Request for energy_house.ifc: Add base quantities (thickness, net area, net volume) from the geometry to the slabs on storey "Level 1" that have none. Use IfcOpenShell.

First a look at what the model holds.

```python
import ifcopenshell
import ifcopenshell.util.element
import ifcopenshell.util.unit

model = ifcopenshell.open("energy_house.ifc")
print(model.schema)
for unit_type in ("LENGTHUNIT", "AREAUNIT", "VOLUMEUNIT"):
    print(unit_type, ifcopenshell.util.unit.calculate_unit_scale(model, unit_type))
storey = next(s for s in model.by_type("IfcBuildingStorey") if s.Name == "Level 1")
slabs = [e for e in ifcopenshell.util.element.get_decomposition(storey) if e.is_a("IfcSlab")]
for e in sorted(slabs, key=lambda e: e.id()):
    print(e.id(), e.is_a(), e.Name, list(ifcopenshell.util.element.get_psets(e, qtos_only=True)), sep=" | ")
```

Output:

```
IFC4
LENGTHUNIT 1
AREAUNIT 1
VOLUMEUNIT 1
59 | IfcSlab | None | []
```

```python
import ifcopenshell
import ifcopenshell.api.pset
import ifcopenshell.geom
import ifcopenshell.util.element
import ifcopenshell.util.shape
import ifcopenshell.util.unit

model = ifcopenshell.open("energy_house.ifc")
unit_scale = ifcopenshell.util.unit.calculate_unit_scale(model)
area_scale = ifcopenshell.util.unit.calculate_unit_scale(model, "AREAUNIT")
volume_scale = ifcopenshell.util.unit.calculate_unit_scale(model, "VOLUMEUNIT")
settings = ifcopenshell.geom.settings()

storey = next(s for s in model.by_type("IfcBuildingStorey") if s.Name == "Level 1")
slabs = [e for e in ifcopenshell.util.element.get_decomposition(storey) if e.is_a("IfcSlab")]

for e in sorted(slabs, key=lambda e: e.id()):
    if ifcopenshell.util.element.get_psets(e, qtos_only=True, should_inherit=False):
        continue
    # Geometry comes back in metres, in the element's own axes.
    shape = ifcopenshell.geom.create_shape(settings, e)
    values = {
        "Width": ifcopenshell.util.shape.get_z(shape.geometry) / unit_scale,
        "NetArea": ifcopenshell.util.shape.get_footprint_area(shape.geometry) / area_scale,
        "NetVolume": ifcopenshell.util.shape.get_volume(shape.geometry) / volume_scale,
    }
    qto = ifcopenshell.api.pset.add_qto(model, product=e, name="Qto_SlabBaseQuantities")
    ifcopenshell.api.pset.edit_qto(model, qto=qto, properties=values)
    print(e.id(), {k: round(v, 3) for k, v in values.items()})

model.write("energy_house_v2.ifc")
```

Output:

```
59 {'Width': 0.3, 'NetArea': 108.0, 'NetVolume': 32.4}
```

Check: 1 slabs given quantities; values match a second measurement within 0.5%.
